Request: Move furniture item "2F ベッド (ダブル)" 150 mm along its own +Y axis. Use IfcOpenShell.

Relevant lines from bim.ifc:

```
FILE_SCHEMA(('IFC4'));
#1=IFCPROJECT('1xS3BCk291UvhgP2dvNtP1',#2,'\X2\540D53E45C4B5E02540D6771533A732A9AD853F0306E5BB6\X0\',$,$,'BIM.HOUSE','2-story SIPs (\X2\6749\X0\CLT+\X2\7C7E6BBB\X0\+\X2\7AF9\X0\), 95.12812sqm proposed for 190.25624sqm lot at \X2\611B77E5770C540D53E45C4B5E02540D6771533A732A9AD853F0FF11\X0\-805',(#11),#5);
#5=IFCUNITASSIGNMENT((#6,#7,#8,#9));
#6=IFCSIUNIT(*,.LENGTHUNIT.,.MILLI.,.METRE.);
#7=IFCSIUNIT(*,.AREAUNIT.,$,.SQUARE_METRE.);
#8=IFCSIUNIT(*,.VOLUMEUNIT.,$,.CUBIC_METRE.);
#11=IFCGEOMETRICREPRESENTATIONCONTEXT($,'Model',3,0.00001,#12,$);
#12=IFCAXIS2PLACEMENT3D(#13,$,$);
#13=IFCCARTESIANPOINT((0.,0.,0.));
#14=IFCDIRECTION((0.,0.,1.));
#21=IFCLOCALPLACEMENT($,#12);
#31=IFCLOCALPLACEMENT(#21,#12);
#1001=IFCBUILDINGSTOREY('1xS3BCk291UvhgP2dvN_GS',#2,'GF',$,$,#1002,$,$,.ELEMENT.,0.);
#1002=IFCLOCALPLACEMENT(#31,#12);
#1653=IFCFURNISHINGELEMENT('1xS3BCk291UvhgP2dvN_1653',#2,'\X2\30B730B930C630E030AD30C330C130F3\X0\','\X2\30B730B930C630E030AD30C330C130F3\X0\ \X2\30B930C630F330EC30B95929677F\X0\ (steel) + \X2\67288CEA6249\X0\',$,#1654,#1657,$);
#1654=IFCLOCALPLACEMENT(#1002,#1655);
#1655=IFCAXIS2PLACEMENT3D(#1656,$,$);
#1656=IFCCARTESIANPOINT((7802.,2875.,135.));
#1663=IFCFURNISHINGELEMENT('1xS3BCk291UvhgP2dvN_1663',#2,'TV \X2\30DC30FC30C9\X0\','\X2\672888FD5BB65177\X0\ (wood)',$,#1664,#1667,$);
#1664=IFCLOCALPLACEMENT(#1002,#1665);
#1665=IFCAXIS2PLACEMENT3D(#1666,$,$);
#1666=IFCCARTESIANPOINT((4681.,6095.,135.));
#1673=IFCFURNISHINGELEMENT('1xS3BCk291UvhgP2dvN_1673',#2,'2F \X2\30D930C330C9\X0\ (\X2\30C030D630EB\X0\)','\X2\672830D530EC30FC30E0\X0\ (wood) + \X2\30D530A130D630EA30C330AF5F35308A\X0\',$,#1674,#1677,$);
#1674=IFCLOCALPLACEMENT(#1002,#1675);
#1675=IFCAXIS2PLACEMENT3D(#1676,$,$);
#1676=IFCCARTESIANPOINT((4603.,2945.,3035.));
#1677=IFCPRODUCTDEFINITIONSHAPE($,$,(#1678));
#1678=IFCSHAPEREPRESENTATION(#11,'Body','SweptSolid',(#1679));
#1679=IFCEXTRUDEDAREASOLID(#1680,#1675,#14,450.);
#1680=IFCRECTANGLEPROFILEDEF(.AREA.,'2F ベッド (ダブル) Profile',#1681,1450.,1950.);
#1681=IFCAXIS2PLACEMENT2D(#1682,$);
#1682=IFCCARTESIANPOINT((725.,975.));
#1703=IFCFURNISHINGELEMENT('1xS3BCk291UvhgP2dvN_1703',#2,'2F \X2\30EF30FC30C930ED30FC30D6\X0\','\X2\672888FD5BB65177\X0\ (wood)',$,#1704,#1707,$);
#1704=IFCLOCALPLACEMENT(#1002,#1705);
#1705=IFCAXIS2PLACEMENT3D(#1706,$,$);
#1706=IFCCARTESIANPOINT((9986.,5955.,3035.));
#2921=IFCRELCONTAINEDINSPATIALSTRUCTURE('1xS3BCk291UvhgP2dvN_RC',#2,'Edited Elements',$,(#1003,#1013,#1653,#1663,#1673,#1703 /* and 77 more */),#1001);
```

```python
import ifcopenshell
import ifcopenshell.api.geometry
import ifcopenshell.util.placement
import ifcopenshell.util.unit

model = ifcopenshell.open("bim.ifc")
unit_scale = ifcopenshell.util.unit.calculate_unit_scale(model)

item = model.by_id(1673)
matrix = ifcopenshell.util.placement.get_local_placement(item.ObjectPlacement)
matrix[:3, 3] += matrix[:3, 1] * 0.15 / unit_scale
ifcopenshell.api.geometry.edit_object_placement(model, product=item, matrix=matrix, is_si=False)

print(ifcopenshell.util.placement.get_local_placement(item.ObjectPlacement).round(3) + 0.0)

model.write("bim-out.ifc")
```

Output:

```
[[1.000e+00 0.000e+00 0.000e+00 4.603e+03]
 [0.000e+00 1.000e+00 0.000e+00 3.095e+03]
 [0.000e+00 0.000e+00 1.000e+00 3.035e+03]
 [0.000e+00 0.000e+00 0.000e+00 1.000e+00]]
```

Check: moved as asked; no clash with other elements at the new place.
